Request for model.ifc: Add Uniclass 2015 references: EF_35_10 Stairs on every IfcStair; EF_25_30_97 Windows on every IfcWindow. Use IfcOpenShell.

First a look at what the model holds.

```python
import ifcopenshell

model = ifcopenshell.open("model.ifc")
print(model.schema)
print("classifications:", [c.Name for c in model.by_type("IfcClassification")])
for ifc_class in ("IfcDoor", "IfcRoof", "IfcStair", "IfcWall", "IfcWindow"):
    print(ifc_class, len(model.by_type(ifc_class)))
```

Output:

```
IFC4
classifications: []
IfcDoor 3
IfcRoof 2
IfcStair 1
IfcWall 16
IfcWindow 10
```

```python
import ifcopenshell
import ifcopenshell.api.classification

model = ifcopenshell.open("model.ifc")

system = ifcopenshell.api.classification.add_classification(model, classification="Uniclass 2015")

codes = {
    "IfcStair": ("EF_35_10", "Stairs"),
    "IfcWindow": ("EF_25_30_97", "Windows"),
}
for ifc_class, (code, name) in codes.items():
    products = model.by_type(ifc_class)
    ifcopenshell.api.classification.add_reference(
        model, products=products, classification=system, identification=code, name=name
    )
    print(code, len(products))

model.write("model_updated.ifc")
```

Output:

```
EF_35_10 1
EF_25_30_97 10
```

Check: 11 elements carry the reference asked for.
